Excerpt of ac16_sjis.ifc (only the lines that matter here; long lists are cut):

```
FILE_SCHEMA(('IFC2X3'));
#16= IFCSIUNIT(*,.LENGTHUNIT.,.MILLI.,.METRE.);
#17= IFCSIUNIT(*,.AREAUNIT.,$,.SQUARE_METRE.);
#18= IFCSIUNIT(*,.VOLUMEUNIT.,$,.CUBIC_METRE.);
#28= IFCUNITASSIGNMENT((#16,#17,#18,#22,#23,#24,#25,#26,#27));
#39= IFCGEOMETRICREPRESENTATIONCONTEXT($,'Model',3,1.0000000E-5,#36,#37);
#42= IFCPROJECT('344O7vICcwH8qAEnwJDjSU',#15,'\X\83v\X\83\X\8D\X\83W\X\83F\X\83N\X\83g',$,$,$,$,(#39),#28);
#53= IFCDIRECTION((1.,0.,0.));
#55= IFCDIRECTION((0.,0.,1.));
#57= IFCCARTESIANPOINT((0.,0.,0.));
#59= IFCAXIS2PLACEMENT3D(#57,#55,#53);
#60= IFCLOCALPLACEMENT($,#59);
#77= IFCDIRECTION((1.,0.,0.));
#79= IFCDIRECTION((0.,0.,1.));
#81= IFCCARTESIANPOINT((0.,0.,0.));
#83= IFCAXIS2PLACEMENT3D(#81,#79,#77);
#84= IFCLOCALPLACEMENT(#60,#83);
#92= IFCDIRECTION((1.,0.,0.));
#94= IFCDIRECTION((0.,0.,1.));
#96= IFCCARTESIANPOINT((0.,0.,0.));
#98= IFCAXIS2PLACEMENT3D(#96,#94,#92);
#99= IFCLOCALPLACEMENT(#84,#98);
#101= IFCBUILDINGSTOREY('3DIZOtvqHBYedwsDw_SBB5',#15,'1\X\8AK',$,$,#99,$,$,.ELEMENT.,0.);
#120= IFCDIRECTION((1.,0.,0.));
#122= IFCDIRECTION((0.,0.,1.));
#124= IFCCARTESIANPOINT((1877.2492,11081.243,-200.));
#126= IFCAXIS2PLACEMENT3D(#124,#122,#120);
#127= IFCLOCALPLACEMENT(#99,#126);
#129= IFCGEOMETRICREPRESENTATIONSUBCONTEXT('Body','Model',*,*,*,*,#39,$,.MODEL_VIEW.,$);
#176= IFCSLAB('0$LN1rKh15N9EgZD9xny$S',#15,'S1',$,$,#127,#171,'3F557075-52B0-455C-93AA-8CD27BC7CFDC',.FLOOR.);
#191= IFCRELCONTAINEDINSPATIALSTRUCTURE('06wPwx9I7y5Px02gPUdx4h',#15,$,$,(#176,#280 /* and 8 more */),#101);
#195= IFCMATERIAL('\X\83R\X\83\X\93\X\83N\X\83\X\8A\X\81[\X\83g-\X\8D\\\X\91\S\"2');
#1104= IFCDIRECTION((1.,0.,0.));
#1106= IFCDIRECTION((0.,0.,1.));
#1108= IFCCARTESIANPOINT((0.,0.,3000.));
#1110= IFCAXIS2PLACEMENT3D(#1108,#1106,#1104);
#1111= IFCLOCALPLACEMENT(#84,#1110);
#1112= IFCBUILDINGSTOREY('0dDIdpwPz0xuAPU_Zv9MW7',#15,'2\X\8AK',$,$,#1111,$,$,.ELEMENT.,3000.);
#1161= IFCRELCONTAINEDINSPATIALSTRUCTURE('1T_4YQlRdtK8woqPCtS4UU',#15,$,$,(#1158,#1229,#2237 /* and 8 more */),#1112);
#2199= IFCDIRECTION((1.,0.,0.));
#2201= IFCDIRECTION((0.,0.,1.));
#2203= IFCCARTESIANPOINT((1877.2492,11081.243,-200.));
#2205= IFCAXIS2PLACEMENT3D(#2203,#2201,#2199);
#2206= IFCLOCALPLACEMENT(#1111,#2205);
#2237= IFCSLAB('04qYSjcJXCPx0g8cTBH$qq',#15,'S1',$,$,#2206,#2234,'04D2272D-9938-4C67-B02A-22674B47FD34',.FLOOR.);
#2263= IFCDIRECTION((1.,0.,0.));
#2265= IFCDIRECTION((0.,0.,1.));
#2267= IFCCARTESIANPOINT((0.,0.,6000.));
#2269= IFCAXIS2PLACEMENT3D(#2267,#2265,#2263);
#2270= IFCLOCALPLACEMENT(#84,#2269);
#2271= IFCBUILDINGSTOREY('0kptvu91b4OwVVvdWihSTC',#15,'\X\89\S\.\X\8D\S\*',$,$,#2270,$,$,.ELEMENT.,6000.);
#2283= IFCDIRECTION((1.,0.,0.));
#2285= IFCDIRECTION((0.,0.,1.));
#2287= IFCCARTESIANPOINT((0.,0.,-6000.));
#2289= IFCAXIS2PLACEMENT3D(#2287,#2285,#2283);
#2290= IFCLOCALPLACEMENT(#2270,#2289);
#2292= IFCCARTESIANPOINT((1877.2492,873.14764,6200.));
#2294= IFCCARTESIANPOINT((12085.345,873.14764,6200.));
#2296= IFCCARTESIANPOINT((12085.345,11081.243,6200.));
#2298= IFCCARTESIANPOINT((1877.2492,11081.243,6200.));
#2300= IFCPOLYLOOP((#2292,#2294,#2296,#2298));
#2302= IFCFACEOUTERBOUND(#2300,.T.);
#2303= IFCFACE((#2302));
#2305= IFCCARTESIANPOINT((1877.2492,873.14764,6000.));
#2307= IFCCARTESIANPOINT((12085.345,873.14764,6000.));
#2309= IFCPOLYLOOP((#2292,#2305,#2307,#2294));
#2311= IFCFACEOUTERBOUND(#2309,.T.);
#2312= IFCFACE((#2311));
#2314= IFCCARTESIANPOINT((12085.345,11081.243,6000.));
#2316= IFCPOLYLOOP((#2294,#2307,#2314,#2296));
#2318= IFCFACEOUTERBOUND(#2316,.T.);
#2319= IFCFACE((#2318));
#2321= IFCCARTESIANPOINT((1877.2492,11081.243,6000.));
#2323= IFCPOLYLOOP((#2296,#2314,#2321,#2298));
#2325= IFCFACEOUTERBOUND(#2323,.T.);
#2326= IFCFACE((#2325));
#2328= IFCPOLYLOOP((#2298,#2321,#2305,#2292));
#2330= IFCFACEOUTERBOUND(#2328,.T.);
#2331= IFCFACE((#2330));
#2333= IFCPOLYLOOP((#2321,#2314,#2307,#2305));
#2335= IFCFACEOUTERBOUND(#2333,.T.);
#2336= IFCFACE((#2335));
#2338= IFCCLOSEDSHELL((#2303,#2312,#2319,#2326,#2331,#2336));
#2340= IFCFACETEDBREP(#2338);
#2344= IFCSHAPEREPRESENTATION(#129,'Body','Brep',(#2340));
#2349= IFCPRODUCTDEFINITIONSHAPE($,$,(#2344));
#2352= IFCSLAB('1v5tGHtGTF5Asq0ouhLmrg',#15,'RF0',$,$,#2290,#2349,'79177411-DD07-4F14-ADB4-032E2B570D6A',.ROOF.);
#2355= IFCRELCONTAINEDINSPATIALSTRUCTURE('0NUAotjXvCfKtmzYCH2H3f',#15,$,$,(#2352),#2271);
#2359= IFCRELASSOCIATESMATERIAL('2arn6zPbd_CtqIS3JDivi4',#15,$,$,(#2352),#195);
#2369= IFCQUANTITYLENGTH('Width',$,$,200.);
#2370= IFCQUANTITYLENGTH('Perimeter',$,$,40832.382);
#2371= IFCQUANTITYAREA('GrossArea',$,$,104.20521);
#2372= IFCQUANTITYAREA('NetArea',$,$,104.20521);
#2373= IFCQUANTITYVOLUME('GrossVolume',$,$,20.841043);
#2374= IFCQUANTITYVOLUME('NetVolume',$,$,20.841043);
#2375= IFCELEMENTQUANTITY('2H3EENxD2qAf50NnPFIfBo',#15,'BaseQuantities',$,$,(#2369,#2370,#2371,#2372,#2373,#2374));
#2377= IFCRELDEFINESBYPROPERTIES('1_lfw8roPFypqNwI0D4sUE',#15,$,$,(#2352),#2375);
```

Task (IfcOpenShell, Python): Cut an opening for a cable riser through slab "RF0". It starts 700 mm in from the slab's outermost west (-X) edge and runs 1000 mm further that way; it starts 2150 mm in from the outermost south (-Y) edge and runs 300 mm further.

```python
import numpy as np
import ifcopenshell
import ifcopenshell.api.feature
import ifcopenshell.api.geometry
import ifcopenshell.api.pset
import ifcopenshell.api.root
import ifcopenshell.geom
import ifcopenshell.util.element
import ifcopenshell.util.placement
import ifcopenshell.util.representation
import ifcopenshell.util.shape
import ifcopenshell.util.unit

model = ifcopenshell.open("ac16_sjis.ifc")
unit_scale = ifcopenshell.util.unit.calculate_unit_scale(model)
area_scale = ifcopenshell.util.unit.calculate_unit_scale(model, "AREAUNIT")
volume_scale = ifcopenshell.util.unit.calculate_unit_scale(model, "VOLUMEUNIT")
settings = ifcopenshell.geom.settings()


def volume(element):
    """Net volume in cubic metres, openings subtracted."""
    shape = ifcopenshell.geom.create_shape(settings, element)
    return ifcopenshell.util.shape.get_volume(shape.geometry)


slab = model.by_guid("1v5tGHtGTF5Asq0ouhLmrg")
before = volume(slab)

# Extent in the slab's own axes, in metres. The edges named are its -X and -Y sides.
slab_shape = ifcopenshell.geom.create_shape(settings, slab)
vertices = ifcopenshell.util.shape.get_vertices(slab_shape.geometry)
x_min, y_min, bottom = vertices.min(axis=0)
top = vertices[:, 2].max()

opening = ifcopenshell.api.root.create_entity(model, ifc_class="IfcOpeningElement", name="Cable riser opening")
context = ifcopenshell.util.representation.get_context(model, "Model", "Body", "MODEL_VIEW")
width, depth = 1, 0.3
outline = [(0.0, 0.0), (width, 0.0), (width, depth), (0.0, depth), (0.0, 0.0)]
# Overshoot both faces by 50 mm so the cut is clean.
shape = ifcopenshell.api.geometry.add_slab_representation(
    model, context=context, depth=top - bottom + 0.1, polyline=outline
)
ifcopenshell.api.geometry.assign_representation(model, product=opening, representation=shape)

matrix = ifcopenshell.util.placement.get_local_placement(slab.ObjectPlacement)
matrix[:, 3] = matrix @ np.append(np.array([x_min + 0.7, y_min + 2.15, bottom - 0.05]) / unit_scale, 1.0)
ifcopenshell.api.geometry.edit_object_placement(model, product=opening, matrix=matrix, is_si=False)
ifcopenshell.api.feature.add_feature(model, feature=opening, element=slab)

after = volume(slab)

# Update the slab's stored quantities.
qto = model.by_id(ifcopenshell.util.element.get_pset(slab, "BaseQuantities", should_inherit=False)["id"])
ifcopenshell.api.pset.edit_qto(model, qto=qto, properties={
    "NetArea": after / (top - bottom) / area_scale,
    "NetVolume": after / volume_scale,
})

print(f"slab volume {before:.3f} -> {after:.3f} m3")

model.write("ac16_sjis_updated.ifc")
```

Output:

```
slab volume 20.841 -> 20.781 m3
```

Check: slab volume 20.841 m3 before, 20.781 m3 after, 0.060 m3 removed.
